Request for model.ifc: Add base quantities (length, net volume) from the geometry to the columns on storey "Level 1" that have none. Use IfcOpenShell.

First a look at what the model holds.

```python
import ifcopenshell
import ifcopenshell.util.element
import ifcopenshell.util.unit

model = ifcopenshell.open("model.ifc")
print(model.schema)
for unit_type in ("LENGTHUNIT", "AREAUNIT", "VOLUMEUNIT"):
    print(unit_type, ifcopenshell.util.unit.calculate_unit_scale(model, unit_type))
storey = next(s for s in model.by_type("IfcBuildingStorey") if s.Name == "Level 1")
columns = [e for e in ifcopenshell.util.element.get_decomposition(storey) if e.is_a("IfcColumn")]
for e in sorted(columns, key=lambda e: e.id()):
    print(e.id(), e.is_a(), e.Name, list(ifcopenshell.util.element.get_psets(e, qtos_only=True)), sep=" | ")
```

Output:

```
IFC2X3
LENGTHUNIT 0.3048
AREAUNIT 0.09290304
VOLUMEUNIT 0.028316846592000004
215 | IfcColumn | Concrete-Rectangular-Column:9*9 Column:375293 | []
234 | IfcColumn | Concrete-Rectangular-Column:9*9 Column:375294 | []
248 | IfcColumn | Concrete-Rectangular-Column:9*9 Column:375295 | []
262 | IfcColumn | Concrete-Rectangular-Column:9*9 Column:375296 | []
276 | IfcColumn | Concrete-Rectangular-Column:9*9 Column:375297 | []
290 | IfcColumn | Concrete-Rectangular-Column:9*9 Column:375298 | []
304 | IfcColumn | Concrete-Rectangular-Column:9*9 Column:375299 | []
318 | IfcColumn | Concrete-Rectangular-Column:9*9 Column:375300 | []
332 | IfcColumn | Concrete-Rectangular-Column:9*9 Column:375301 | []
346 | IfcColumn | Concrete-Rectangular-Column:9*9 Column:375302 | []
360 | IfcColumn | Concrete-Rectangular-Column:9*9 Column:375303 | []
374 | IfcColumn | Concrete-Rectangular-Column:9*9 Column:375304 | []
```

```python
import ifcopenshell
import ifcopenshell.api.pset
import ifcopenshell.geom
import ifcopenshell.util.element
import ifcopenshell.util.shape
import ifcopenshell.util.unit

model = ifcopenshell.open("model.ifc")
unit_scale = ifcopenshell.util.unit.calculate_unit_scale(model)
volume_scale = ifcopenshell.util.unit.calculate_unit_scale(model, "VOLUMEUNIT")
settings = ifcopenshell.geom.settings()

storey = next(s for s in model.by_type("IfcBuildingStorey") if s.Name == "Level 1")
columns = [e for e in ifcopenshell.util.element.get_decomposition(storey) if e.is_a("IfcColumn")]

for e in sorted(columns, key=lambda e: e.id()):
    if ifcopenshell.util.element.get_psets(e, qtos_only=True, should_inherit=False):
        continue
    # Geometry comes back in metres, in the element's own axes.
    shape = ifcopenshell.geom.create_shape(settings, e)
    values = {
        "Length": ifcopenshell.util.shape.get_z(shape.geometry) / unit_scale,
        "NetVolume": ifcopenshell.util.shape.get_volume(shape.geometry) / volume_scale,
    }
    qto = ifcopenshell.api.pset.add_qto(model, product=e, name="BaseQuantities")
    ifcopenshell.api.pset.edit_qto(model, qto=qto, properties=values)
    print(e.id(), {k: round(v, 3) for k, v in values.items()})

model.write("model_rev.ifc")
```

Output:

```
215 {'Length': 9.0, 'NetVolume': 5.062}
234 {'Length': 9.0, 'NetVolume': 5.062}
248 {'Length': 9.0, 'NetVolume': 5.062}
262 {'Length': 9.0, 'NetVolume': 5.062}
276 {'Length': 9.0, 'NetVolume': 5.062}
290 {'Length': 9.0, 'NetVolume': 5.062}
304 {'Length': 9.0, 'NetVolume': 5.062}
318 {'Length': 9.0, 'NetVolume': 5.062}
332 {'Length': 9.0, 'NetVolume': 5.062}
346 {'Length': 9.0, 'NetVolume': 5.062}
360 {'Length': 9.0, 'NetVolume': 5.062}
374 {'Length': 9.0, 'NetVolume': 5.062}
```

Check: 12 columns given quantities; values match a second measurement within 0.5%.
